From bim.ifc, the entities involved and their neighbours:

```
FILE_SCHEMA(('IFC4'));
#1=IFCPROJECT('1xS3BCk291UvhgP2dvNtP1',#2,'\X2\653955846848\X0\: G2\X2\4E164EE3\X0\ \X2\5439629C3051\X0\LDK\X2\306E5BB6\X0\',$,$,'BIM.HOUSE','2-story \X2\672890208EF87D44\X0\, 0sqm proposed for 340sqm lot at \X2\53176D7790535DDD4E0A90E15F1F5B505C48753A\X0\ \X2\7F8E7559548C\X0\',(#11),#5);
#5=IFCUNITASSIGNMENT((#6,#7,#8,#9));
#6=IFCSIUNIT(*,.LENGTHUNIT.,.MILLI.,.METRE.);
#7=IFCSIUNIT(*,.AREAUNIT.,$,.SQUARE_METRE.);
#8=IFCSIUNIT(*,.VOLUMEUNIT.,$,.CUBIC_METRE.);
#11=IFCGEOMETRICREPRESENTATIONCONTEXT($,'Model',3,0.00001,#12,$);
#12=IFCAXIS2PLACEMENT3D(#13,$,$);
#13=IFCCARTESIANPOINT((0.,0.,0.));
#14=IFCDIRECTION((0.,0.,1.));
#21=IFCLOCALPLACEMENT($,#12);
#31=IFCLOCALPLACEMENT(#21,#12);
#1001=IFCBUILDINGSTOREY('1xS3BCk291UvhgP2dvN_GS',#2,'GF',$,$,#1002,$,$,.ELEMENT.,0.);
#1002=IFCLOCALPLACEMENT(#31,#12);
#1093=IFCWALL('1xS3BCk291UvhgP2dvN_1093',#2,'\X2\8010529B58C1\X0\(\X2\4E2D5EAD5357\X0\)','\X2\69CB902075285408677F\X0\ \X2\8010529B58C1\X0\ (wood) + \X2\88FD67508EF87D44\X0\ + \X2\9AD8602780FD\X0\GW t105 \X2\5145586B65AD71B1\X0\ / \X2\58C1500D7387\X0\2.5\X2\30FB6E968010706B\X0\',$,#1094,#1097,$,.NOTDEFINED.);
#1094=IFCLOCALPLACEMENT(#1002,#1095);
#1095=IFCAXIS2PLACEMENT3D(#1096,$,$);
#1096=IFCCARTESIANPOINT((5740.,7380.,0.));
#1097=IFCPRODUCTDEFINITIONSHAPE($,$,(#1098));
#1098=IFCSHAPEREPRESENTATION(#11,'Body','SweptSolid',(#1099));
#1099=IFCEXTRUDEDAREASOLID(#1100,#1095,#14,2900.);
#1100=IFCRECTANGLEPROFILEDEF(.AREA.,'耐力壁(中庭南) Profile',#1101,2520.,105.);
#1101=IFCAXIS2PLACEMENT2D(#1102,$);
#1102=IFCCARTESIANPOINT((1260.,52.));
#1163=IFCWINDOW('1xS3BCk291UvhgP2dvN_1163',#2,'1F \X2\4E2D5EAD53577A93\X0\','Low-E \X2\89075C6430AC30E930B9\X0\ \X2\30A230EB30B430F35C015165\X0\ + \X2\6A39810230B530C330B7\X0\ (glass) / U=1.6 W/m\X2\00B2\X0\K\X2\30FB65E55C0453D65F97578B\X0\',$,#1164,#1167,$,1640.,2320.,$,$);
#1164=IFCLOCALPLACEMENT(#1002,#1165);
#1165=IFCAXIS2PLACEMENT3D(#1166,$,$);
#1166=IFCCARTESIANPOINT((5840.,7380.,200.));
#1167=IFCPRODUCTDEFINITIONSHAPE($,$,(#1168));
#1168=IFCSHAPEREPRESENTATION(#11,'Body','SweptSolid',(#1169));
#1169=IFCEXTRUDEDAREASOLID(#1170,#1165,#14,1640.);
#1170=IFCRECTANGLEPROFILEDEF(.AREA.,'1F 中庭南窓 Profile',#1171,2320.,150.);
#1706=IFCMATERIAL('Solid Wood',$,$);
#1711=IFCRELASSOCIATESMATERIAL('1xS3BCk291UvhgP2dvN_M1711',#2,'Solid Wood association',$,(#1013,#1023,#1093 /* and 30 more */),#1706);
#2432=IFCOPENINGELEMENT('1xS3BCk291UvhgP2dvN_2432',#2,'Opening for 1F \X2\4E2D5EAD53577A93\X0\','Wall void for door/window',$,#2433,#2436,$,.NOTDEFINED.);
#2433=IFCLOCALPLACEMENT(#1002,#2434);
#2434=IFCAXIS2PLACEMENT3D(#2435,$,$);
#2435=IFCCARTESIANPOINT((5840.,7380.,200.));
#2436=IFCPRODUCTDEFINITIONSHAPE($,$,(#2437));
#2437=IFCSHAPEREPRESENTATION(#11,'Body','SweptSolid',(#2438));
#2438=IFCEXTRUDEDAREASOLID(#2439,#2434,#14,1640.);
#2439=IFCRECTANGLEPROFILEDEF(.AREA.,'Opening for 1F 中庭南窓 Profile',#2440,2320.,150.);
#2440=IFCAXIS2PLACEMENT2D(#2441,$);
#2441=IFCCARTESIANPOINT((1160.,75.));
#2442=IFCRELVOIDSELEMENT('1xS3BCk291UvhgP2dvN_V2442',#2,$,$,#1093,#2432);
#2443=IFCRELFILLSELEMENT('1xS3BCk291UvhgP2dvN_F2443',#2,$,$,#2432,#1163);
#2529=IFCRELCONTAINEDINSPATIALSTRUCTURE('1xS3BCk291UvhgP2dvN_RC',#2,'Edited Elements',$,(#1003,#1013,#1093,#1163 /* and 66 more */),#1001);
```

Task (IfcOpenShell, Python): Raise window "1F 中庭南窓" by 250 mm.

```python
import numpy as np
import ifcopenshell
import ifcopenshell.api.geometry
import ifcopenshell.util.placement
import ifcopenshell.util.unit

model = ifcopenshell.open("bim.ifc")
unit_scale = ifcopenshell.util.unit.calculate_unit_scale(model)

window = model.by_id(1163)
opening = window.FillsVoids[0].RelatingOpeningElement
dz = 0.25 / unit_scale

shift = np.array([0.0, 0.0, dz])
# The window is not placed relative to its opening, so move both.
for product in (opening, window):
    matrix = ifcopenshell.util.placement.get_local_placement(product.ObjectPlacement)
    matrix[:3, 3] += shift
    ifcopenshell.api.geometry.edit_object_placement(model, product=product, matrix=matrix, is_si=False)

print(f"moved by {dz * unit_scale:+.3f} m")

model.write("bim_edited.ifc")
```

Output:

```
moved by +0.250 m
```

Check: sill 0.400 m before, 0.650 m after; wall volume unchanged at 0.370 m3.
